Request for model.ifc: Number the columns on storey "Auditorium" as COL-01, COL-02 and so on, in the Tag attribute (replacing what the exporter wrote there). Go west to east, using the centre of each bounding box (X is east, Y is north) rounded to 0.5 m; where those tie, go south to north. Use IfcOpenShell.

First a look at what the model holds.

```python
import ifcopenshell
import ifcopenshell.util.element
import ifcopenshell.util.placement

model = ifcopenshell.open("model.ifc")
print(model.schema)
storey = next(s for s in model.by_type("IfcBuildingStorey") if s.Name == "Auditorium")
columns = [e for e in ifcopenshell.util.element.get_decomposition(storey) if e.is_a("IfcColumn")]
for e in sorted(columns, key=lambda e: e.id()):
    origin = ifcopenshell.util.placement.get_local_placement(e.ObjectPlacement)[:3, 3]
    print(e.id(), e.Tag, e.Name, origin.round(2) + 0.0, sep=" | ")
```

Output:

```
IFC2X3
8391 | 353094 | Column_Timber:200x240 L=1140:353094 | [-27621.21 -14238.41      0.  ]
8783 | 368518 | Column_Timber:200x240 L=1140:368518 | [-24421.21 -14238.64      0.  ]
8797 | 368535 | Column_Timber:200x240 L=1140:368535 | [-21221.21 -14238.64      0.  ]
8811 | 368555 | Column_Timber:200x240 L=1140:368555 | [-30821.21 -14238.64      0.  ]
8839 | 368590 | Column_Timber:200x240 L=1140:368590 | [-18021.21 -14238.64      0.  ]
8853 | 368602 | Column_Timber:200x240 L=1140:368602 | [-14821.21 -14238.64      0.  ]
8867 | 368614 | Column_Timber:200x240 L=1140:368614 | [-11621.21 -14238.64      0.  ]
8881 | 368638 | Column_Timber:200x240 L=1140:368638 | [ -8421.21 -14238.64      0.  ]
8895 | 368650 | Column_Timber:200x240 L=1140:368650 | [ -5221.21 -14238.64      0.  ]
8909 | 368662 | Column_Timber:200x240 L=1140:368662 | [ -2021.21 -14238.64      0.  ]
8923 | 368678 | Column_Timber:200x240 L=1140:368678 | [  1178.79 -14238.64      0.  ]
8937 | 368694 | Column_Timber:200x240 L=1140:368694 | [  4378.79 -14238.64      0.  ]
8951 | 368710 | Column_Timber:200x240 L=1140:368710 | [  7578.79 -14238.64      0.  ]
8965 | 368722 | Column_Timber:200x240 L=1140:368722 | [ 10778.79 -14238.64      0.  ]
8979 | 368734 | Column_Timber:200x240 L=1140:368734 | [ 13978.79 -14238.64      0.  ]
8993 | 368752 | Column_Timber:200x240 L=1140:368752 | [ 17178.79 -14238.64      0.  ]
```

```python
import ifcopenshell
import ifcopenshell.geom
import ifcopenshell.util.element
import ifcopenshell.util.shape

model = ifcopenshell.open("model.ifc")
settings = ifcopenshell.geom.settings()
settings.set("use-world-coords", True)


def centre(element):
    shape = ifcopenshell.geom.create_shape(settings, element)
    return ifcopenshell.util.shape.get_bbox_centroid(shape.geometry)


storey = next(s for s in model.by_type("IfcBuildingStorey") if s.Name == "Auditorium")
columns = [e for e in ifcopenshell.util.element.get_decomposition(storey) if e.is_a("IfcColumn")]

# Insertion points can sit at a corner or the storey origin, so sort by the geometry (in metres).
centres = {e: centre(e) for e in columns}
columns.sort(key=lambda e: (round(centres[e][0] / 0.5), centres[e][1]))

for i, e in enumerate(columns, start=1):
    number = f"COL-{i:02d}"
    e.Tag = number
    print(e.id(), number)

model.write("model-out.ifc")
```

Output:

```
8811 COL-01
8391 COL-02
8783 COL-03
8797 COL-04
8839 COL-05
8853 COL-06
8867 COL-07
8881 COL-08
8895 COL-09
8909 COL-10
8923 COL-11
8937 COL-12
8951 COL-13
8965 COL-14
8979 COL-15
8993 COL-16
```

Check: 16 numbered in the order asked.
